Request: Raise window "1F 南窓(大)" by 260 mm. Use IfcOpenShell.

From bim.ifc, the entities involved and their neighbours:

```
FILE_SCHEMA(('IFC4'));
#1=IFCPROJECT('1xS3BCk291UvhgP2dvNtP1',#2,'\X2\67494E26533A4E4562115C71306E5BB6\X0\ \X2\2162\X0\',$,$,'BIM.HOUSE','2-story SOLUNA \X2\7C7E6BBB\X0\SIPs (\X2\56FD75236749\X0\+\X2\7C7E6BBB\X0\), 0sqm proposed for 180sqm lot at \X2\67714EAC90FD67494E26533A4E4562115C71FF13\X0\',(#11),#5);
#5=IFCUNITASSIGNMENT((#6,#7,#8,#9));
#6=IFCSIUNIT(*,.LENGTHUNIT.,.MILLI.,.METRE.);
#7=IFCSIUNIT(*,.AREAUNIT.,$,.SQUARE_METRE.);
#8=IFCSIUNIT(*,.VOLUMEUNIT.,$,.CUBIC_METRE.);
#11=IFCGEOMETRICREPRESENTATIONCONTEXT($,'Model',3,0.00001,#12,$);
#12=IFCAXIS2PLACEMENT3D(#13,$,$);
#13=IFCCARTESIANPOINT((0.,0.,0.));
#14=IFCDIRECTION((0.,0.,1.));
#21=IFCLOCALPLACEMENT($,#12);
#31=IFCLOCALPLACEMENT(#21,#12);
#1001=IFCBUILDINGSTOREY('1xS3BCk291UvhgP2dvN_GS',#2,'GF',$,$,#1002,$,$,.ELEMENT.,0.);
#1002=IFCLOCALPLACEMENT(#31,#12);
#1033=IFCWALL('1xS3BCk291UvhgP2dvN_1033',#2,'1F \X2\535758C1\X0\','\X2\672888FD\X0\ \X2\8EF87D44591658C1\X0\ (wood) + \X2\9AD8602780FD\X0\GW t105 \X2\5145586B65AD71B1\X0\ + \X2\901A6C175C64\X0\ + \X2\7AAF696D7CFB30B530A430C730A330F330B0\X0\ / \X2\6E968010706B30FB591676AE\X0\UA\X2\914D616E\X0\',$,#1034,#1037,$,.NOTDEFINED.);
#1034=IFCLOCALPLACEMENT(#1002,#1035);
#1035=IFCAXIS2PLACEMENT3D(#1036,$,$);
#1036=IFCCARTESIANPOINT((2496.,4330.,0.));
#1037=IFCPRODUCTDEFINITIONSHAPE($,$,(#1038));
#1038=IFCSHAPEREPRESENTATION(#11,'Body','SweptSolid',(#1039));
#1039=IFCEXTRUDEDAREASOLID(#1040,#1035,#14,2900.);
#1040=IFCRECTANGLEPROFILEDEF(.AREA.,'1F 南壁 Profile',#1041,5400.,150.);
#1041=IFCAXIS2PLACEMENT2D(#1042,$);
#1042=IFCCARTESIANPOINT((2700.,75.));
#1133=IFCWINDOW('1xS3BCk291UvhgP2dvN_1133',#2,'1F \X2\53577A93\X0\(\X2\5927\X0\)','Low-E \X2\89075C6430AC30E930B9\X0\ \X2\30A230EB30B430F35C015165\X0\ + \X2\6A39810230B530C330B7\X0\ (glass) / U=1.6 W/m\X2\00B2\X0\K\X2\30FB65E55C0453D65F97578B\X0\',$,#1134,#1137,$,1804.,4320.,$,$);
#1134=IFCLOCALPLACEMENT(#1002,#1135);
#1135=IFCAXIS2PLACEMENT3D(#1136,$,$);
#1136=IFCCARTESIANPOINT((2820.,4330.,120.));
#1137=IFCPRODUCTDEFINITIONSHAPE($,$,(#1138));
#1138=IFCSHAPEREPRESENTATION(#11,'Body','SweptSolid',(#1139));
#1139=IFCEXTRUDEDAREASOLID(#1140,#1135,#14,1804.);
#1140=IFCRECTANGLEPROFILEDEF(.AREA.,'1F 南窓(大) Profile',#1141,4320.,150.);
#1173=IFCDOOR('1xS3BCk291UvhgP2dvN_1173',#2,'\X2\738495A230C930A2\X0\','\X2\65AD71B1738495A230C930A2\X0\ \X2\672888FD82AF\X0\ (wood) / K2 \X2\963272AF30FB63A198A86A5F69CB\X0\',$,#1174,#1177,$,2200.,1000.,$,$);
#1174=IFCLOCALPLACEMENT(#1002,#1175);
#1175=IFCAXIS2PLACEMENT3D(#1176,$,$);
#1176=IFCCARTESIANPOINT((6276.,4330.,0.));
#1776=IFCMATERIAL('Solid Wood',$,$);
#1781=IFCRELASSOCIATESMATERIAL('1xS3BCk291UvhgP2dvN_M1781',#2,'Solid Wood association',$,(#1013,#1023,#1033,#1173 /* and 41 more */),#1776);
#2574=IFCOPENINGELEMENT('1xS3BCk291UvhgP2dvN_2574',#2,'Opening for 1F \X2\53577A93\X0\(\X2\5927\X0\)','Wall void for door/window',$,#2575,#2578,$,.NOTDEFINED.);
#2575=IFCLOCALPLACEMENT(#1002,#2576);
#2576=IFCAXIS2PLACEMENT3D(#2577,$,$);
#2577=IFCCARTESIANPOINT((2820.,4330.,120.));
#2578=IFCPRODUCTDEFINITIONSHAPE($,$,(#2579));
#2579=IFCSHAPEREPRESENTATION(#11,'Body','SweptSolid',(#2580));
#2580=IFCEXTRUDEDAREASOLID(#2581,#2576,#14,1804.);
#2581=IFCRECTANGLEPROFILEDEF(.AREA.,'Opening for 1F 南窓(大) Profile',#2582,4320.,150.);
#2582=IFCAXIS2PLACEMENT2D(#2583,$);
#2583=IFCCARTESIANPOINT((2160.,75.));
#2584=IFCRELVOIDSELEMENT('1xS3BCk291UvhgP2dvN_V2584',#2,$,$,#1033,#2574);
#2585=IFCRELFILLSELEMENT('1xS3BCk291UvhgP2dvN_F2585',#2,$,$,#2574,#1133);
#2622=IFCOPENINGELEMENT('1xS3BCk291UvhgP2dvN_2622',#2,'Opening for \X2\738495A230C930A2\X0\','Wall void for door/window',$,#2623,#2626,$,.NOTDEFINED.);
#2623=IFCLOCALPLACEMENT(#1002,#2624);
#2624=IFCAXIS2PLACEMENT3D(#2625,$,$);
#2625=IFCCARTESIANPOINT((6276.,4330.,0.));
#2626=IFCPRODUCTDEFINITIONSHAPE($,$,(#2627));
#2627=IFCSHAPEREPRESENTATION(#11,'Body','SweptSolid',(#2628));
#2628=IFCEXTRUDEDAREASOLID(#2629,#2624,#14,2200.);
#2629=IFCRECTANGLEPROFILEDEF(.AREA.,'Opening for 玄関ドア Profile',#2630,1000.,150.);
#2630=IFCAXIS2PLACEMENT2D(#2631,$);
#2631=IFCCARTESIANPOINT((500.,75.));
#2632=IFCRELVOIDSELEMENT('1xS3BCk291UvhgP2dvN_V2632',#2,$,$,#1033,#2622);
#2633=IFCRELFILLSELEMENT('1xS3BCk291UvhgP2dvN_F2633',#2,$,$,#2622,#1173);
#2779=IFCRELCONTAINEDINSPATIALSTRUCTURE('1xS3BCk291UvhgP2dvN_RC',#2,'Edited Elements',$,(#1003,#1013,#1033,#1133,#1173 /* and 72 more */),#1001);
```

```python
import numpy as np
import ifcopenshell
import ifcopenshell.api.geometry
import ifcopenshell.util.placement
import ifcopenshell.util.unit

model = ifcopenshell.open("bim.ifc")
unit_scale = ifcopenshell.util.unit.calculate_unit_scale(model)

window = model.by_id(1133)
opening = window.FillsVoids[0].RelatingOpeningElement
dz = 0.26 / unit_scale

shift = np.array([0.0, 0.0, dz])
# The window is not placed relative to its opening, so move both.
for product in (opening, window):
    matrix = ifcopenshell.util.placement.get_local_placement(product.ObjectPlacement)
    matrix[:3, 3] += shift
    ifcopenshell.api.geometry.edit_object_placement(model, product=product, matrix=matrix, is_si=False)

print(f"moved by {dz * unit_scale:+.3f} m")

model.write("bim_rev.ifc")
```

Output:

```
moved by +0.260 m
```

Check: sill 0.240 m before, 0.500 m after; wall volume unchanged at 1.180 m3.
